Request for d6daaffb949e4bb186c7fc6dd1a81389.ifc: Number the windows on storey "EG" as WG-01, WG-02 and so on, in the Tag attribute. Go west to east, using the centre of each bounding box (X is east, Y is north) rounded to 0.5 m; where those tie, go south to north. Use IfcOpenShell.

First a look at what the model holds.

```python
import ifcopenshell
import ifcopenshell.util.element
import ifcopenshell.util.placement

model = ifcopenshell.open("d6daaffb949e4bb186c7fc6dd1a81389.ifc")
print(model.schema)
storey = next(s for s in model.by_type("IfcBuildingStorey") if s.Name == "EG")
windows = [e for e in ifcopenshell.util.element.get_decomposition(storey) if e.is_a("IfcWindow")]
for e in sorted(windows, key=lambda e: e.id()):
    origin = ifcopenshell.util.placement.get_local_placement(e.ObjectPlacement)[:3, 3]
    print(e.id(), e.Tag, e.Name, origin.round(2) + 0.0, sep=" | ")
```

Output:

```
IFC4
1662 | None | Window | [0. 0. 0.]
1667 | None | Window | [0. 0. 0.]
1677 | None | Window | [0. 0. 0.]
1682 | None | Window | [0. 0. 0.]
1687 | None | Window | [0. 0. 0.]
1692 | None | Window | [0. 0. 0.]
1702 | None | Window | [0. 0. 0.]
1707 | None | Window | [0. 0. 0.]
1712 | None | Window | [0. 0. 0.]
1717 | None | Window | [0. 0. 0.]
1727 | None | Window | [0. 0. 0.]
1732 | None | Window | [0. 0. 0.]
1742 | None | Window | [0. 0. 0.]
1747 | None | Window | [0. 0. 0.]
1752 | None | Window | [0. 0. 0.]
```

```python
import ifcopenshell
import ifcopenshell.geom
import ifcopenshell.util.element
import ifcopenshell.util.shape

model = ifcopenshell.open("d6daaffb949e4bb186c7fc6dd1a81389.ifc")
settings = ifcopenshell.geom.settings()
settings.set("use-world-coords", True)


def centre(element):
    shape = ifcopenshell.geom.create_shape(settings, element)
    return ifcopenshell.util.shape.get_bbox_centroid(shape.geometry)


storey = next(s for s in model.by_type("IfcBuildingStorey") if s.Name == "EG")
windows = [e for e in ifcopenshell.util.element.get_decomposition(storey) if e.is_a("IfcWindow")]

# Insertion points can sit at a corner or the storey origin, so sort by the geometry (in metres).
centres = {e: centre(e) for e in windows}
windows.sort(key=lambda e: (round(centres[e][0] / 0.5), centres[e][1]))

for i, e in enumerate(windows, start=1):
    number = f"WG-{i:02d}"
    e.Tag = number
    print(e.id(), number)

model.write("d6daaffb949e4bb186c7fc6dd1a81389_v2.ifc")
```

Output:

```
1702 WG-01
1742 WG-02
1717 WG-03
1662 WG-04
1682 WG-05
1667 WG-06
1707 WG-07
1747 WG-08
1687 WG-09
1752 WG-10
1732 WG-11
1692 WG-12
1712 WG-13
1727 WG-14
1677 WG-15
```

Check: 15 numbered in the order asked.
